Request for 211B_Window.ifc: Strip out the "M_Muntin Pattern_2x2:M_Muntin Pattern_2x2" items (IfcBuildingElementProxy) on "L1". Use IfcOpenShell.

First a look at what the model holds.

```python
import ifcopenshell
import ifcopenshell.util.element

model = ifcopenshell.open("211B_Window.ifc")
print(model.schema)
storey = next(s for s in model.by_type("IfcBuildingStorey") if s.Name == "L1")
proxies = [e for e in ifcopenshell.util.element.get_decomposition(storey) if e.is_a("IfcBuildingElementProxy")]
seen = {}
for e in proxies:
    element_type = ifcopenshell.util.element.get_type(e)
    name = element_type.Name if element_type not in (None, e) else None
    seen[name] = seen.get(name, 0) + 1
for name, count in sorted(seen.items(), key=str):
    print(count, "x", name)
```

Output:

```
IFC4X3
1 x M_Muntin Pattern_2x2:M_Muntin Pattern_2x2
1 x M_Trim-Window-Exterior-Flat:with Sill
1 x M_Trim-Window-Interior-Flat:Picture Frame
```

```python
import ifcopenshell
import ifcopenshell.api.root
import ifcopenshell.util.element

model = ifcopenshell.open("211B_Window.ifc")

storey = next(s for s in model.by_type("IfcBuildingStorey") if s.Name == "L1")
proxies = [e for e in ifcopenshell.util.element.get_decomposition(storey) if e.is_a("IfcBuildingElementProxy")]
targets = [e for e in proxies if (t := ifcopenshell.util.element.get_type(e)) not in (None, e) and t.Name == "M_Muntin Pattern_2x2:M_Muntin Pattern_2x2"]

for e in targets:
    ifcopenshell.api.root.remove_product(model, product=e)
print(len(targets), "removed")

model.write("211B_Window_updated.ifc")
```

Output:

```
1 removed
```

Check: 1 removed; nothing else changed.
